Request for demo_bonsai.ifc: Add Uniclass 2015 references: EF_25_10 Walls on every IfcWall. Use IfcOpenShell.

First a look at what the model holds.

```python
import ifcopenshell

model = ifcopenshell.open("demo_bonsai.ifc")
print(model.schema)
print("classifications:", [c.Name for c in model.by_type("IfcClassification")])
for ifc_class in ("IfcDoor", "IfcRoof", "IfcStair", "IfcWall", "IfcWindow"):
    print(ifc_class, len(model.by_type(ifc_class)))
```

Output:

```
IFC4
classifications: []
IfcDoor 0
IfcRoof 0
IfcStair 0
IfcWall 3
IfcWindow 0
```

```python
import ifcopenshell
import ifcopenshell.api.classification

model = ifcopenshell.open("demo_bonsai.ifc")

system = ifcopenshell.api.classification.add_classification(model, classification="Uniclass 2015")

codes = {
    "IfcWall": ("EF_25_10", "Walls"),
}
for ifc_class, (code, name) in codes.items():
    products = model.by_type(ifc_class)
    ifcopenshell.api.classification.add_reference(
        model, products=products, classification=system, identification=code, name=name
    )
    print(code, len(products))

model.write("demo_bonsai_v2.ifc")
```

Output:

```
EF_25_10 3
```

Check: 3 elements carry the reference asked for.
